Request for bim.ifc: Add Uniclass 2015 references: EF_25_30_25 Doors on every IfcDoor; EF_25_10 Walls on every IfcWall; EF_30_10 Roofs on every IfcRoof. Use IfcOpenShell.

First a look at what the model holds.

```python
import ifcopenshell

model = ifcopenshell.open("bim.ifc")
print(model.schema)
print("classifications:", [c.Name for c in model.by_type("IfcClassification")])
for ifc_class in ("IfcDoor", "IfcRoof", "IfcStair", "IfcWall", "IfcWindow"):
    print(ifc_class, len(model.by_type(ifc_class)))
```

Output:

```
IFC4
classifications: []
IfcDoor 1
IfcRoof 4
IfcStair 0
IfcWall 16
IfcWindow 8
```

```python
import ifcopenshell
import ifcopenshell.api.classification

model = ifcopenshell.open("bim.ifc")

system = ifcopenshell.api.classification.add_classification(model, classification="Uniclass 2015")

codes = {
    "IfcDoor": ("EF_25_30_25", "Doors"),
    "IfcWall": ("EF_25_10", "Walls"),
    "IfcRoof": ("EF_30_10", "Roofs"),
}
for ifc_class, (code, name) in codes.items():
    products = model.by_type(ifc_class)
    ifcopenshell.api.classification.add_reference(
        model, products=products, classification=system, identification=code, name=name
    )
    print(code, len(products))

model.write("bim_v2.ifc")
```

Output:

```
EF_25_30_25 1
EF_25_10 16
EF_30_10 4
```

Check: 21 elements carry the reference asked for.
